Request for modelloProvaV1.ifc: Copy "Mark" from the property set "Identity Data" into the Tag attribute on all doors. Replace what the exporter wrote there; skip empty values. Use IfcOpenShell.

First a look at what the model holds.

```python
import ifcopenshell
import ifcopenshell.util.element

model = ifcopenshell.open("modelloProvaV1.ifc")
print(model.schema)
doors = model.by_type("IfcDoor")
print(len(doors), "doors")
for e in doors[:8]:
    source = ifcopenshell.util.element.get_pset(e, "Identity Data", "Mark")
    target = e.Tag
    print(e.id(), repr(source), repr(target), sep=" | ")
```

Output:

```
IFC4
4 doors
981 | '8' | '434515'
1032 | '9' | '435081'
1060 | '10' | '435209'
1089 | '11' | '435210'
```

```python
import ifcopenshell
import ifcopenshell.util.element

model = ifcopenshell.open("modelloProvaV1.ifc")

count = 0
for e in model.by_type("IfcDoor"):
    value = ifcopenshell.util.element.get_pset(e, "Identity Data", "Mark")
    current = e.Tag
    if not value or not value.strip() or current == value:
        continue
    e.Tag = value
    count += 1

print(count, "doors updated")

model.write("modelloProvaV1_edited.ifc")
```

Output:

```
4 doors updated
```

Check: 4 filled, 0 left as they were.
